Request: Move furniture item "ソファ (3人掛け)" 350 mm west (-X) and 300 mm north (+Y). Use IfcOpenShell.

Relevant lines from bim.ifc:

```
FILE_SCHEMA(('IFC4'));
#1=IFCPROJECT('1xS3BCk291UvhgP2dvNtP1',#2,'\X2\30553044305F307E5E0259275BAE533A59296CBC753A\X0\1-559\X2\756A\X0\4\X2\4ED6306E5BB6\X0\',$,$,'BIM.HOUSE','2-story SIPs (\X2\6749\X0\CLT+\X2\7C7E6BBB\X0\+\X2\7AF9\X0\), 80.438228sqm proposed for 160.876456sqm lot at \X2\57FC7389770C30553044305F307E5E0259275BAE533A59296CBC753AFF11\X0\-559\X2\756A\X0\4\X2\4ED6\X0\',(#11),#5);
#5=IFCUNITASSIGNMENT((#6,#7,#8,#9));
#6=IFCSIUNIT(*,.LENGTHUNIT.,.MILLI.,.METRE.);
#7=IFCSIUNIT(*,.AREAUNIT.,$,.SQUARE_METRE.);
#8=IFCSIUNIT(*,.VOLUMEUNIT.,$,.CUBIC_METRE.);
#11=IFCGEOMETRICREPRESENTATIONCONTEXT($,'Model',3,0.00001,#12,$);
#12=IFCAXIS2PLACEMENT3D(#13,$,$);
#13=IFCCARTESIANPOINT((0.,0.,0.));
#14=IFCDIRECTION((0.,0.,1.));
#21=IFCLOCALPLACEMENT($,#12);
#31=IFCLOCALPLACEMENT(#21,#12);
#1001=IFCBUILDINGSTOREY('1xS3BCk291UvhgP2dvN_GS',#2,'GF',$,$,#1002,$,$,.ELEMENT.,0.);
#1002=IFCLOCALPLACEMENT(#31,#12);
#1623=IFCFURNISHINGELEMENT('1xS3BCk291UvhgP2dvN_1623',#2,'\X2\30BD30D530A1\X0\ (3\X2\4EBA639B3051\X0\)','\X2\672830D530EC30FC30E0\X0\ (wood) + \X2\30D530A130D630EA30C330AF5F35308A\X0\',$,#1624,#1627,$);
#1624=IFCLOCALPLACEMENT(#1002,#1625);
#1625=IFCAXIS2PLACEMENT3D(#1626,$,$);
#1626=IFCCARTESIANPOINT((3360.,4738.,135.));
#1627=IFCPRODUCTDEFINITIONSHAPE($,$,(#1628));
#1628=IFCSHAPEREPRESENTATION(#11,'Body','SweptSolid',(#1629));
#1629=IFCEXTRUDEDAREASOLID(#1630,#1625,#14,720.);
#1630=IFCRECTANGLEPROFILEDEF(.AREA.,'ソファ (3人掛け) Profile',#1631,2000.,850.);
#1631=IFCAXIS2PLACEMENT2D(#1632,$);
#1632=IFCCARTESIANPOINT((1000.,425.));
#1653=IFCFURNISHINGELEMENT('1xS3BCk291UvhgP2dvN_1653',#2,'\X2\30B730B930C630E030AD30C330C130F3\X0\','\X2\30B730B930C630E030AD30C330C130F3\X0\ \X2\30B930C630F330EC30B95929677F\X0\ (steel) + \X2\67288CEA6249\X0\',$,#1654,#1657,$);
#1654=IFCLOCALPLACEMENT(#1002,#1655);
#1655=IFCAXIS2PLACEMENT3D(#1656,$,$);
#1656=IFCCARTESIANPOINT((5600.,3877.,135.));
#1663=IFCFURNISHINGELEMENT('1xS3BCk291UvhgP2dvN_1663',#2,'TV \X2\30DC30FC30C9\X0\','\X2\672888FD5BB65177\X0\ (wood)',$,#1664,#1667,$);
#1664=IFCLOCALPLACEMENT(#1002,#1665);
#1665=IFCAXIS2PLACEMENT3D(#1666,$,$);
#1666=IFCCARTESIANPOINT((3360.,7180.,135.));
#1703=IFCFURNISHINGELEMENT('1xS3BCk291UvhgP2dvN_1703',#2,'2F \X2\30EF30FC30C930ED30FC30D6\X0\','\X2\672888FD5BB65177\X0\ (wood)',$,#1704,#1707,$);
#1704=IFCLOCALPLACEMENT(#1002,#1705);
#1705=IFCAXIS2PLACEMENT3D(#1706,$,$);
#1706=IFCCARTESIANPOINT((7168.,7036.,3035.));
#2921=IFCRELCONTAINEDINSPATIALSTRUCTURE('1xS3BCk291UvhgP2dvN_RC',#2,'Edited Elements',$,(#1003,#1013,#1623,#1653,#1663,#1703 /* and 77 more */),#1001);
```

```python
import ifcopenshell
import ifcopenshell.api.geometry
import ifcopenshell.util.placement
import ifcopenshell.util.unit

model = ifcopenshell.open("bim.ifc")
unit_scale = ifcopenshell.util.unit.calculate_unit_scale(model)

item = model.by_guid("1xS3BCk291UvhgP2dvN_1623")
matrix = ifcopenshell.util.placement.get_local_placement(item.ObjectPlacement)
matrix[0, 3] -= 0.35 / unit_scale
matrix[1, 3] += 0.3 / unit_scale
ifcopenshell.api.geometry.edit_object_placement(model, product=item, matrix=matrix, is_si=False)

print(ifcopenshell.util.placement.get_local_placement(item.ObjectPlacement).round(3) + 0.0)

model.write("bim-out.ifc")
```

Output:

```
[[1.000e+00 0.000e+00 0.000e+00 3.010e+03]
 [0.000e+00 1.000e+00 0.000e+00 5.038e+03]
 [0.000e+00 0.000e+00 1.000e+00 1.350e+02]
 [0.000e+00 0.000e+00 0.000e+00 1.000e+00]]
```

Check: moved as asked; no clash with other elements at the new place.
